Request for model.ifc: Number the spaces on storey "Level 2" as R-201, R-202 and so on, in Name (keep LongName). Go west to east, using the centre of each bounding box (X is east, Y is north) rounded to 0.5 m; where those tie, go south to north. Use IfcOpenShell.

First a look at what the model holds.

```python
import ifcopenshell
import ifcopenshell.util.element
import ifcopenshell.util.placement

model = ifcopenshell.open("model.ifc")
print(model.schema)
storey = next(s for s in model.by_type("IfcBuildingStorey") if s.Name == "Level 2")
spaces = [e for e in ifcopenshell.util.element.get_decomposition(storey) if e.is_a("IfcSpace")]
for e in sorted(spaces, key=lambda e: e.id()):
    origin = ifcopenshell.util.placement.get_local_placement(e.ObjectPlacement)[:3, 3]
    print(e.id(), e.Name, e.LongName, origin.round(2) + 0.0, sep=" | ")
```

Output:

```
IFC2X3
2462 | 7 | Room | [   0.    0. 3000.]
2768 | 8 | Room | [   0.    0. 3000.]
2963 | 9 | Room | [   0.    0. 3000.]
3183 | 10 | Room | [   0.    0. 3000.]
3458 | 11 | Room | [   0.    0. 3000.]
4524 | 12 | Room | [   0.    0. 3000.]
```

```python
import ifcopenshell
import ifcopenshell.geom
import ifcopenshell.util.element
import ifcopenshell.util.shape

model = ifcopenshell.open("model.ifc")
settings = ifcopenshell.geom.settings()
settings.set("use-world-coords", True)


def centre(element):
    shape = ifcopenshell.geom.create_shape(settings, element)
    return ifcopenshell.util.shape.get_bbox_centroid(shape.geometry)


storey = next(s for s in model.by_type("IfcBuildingStorey") if s.Name == "Level 2")
spaces = [e for e in ifcopenshell.util.element.get_decomposition(storey) if e.is_a("IfcSpace")]

# Insertion points can sit at a corner or the storey origin, so sort by the geometry (in metres).
centres = {e: centre(e) for e in spaces}
spaces.sort(key=lambda e: (round(centres[e][0] / 0.5), centres[e][1]))

for i, e in enumerate(spaces, start=1):
    number = f"R-2{i:02d}"
    e.Name = number
    print(e.id(), number)

model.write("model_rev.ifc")
```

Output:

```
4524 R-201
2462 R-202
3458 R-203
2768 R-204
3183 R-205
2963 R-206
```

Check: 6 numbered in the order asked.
